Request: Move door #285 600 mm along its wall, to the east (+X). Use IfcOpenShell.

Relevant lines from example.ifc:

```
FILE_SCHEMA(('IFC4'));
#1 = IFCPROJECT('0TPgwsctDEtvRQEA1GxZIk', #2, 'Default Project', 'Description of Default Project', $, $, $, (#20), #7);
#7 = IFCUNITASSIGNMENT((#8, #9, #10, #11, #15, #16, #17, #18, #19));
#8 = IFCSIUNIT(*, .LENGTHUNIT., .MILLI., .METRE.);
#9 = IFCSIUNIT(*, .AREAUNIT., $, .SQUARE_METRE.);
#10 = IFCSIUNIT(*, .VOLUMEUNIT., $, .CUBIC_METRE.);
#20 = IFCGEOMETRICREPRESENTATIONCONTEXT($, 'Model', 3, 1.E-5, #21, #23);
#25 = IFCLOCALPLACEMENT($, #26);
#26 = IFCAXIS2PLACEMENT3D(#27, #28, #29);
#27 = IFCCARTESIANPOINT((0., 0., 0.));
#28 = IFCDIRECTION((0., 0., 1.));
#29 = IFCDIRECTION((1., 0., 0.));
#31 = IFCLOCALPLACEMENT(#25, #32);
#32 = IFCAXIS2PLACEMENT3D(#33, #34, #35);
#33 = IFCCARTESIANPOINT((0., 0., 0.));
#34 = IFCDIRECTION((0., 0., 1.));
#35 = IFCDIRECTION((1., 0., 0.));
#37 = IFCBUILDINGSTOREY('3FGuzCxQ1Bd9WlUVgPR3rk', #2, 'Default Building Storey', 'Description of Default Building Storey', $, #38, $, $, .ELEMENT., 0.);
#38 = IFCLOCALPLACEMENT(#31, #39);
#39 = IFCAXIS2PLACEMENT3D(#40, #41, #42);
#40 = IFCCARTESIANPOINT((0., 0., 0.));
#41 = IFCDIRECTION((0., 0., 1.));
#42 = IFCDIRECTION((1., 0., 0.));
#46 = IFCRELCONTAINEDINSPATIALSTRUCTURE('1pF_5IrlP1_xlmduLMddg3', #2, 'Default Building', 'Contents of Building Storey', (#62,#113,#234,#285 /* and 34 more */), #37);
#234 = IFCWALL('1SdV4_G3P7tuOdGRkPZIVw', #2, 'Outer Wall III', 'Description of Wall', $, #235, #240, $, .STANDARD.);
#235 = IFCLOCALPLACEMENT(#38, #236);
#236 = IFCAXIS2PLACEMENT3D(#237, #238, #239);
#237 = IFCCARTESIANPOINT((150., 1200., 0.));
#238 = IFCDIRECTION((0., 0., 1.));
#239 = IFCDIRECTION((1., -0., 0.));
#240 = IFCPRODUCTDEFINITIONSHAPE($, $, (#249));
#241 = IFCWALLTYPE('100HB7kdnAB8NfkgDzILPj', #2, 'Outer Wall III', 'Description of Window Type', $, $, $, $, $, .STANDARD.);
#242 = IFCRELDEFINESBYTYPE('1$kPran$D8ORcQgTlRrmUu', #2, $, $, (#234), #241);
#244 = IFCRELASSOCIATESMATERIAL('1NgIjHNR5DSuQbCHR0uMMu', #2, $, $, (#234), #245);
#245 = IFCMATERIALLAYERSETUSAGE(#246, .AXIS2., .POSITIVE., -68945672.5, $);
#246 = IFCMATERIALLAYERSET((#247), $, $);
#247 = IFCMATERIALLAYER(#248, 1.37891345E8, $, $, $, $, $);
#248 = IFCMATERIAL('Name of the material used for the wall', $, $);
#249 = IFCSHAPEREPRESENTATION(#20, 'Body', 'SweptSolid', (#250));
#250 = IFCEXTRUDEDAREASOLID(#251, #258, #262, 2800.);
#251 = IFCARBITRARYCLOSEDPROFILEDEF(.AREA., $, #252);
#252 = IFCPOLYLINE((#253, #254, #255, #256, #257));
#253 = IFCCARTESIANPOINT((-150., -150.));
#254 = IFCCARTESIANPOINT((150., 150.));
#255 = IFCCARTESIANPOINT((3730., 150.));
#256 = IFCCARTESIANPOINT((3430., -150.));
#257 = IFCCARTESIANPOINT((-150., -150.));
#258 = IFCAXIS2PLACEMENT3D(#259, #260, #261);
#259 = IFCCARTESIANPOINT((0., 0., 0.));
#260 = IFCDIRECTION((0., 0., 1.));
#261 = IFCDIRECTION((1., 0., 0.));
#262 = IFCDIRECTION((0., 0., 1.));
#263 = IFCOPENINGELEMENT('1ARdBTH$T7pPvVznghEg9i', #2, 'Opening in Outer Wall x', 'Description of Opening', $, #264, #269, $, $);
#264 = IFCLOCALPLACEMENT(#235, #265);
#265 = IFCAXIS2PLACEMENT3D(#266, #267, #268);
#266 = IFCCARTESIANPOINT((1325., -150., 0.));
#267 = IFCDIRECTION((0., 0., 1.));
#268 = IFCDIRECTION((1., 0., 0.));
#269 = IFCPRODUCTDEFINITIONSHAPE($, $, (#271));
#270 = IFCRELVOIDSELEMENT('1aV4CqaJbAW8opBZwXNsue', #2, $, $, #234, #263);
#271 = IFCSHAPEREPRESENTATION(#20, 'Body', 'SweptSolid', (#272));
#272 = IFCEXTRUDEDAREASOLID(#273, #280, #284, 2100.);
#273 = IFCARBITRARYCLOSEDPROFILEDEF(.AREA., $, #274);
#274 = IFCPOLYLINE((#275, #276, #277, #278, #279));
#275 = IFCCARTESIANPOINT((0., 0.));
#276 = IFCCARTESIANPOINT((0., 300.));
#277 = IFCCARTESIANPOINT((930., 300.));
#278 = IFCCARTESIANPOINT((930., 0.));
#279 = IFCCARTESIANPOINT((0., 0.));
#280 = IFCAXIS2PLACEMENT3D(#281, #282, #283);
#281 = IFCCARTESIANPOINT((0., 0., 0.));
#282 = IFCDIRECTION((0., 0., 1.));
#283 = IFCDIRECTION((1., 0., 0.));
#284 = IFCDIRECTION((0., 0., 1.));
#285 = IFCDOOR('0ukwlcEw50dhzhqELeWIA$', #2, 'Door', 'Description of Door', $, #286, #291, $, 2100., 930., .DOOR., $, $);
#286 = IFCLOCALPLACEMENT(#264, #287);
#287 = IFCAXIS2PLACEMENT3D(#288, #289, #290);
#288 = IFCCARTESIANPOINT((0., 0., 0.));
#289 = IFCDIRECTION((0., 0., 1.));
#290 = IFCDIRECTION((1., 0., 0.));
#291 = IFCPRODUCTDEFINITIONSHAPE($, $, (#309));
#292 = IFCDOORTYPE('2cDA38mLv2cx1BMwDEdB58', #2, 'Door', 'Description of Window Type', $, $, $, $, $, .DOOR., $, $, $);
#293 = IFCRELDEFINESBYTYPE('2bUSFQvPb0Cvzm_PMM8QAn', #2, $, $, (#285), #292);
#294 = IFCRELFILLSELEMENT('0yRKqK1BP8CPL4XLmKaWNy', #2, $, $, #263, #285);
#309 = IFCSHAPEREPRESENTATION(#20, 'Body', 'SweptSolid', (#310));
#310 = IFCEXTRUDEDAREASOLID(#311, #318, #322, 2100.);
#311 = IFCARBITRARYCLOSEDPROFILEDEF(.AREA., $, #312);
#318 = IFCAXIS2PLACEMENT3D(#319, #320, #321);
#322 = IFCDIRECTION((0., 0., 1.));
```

```python
import ifcopenshell
import ifcopenshell.api.geometry
import ifcopenshell.util.placement
import ifcopenshell.util.unit

model = ifcopenshell.open("example.ifc")
unit_scale = ifcopenshell.util.unit.calculate_unit_scale(model)

door = model.by_id(285)
opening = door.FillsVoids[0].RelatingOpeningElement
wall = opening.VoidsElements[0].RelatingBuildingElement

wall_matrix = ifcopenshell.util.placement.get_local_placement(wall.ObjectPlacement)
shift = wall_matrix[:3, 0] * 0.6 / unit_scale
before = ifcopenshell.util.placement.get_local_placement(door.ObjectPlacement)[:3, 3].copy()

# The door is placed relative to its opening, so it follows when the opening moves.
matrix = ifcopenshell.util.placement.get_local_placement(opening.ObjectPlacement)
matrix[:3, 3] += shift
ifcopenshell.api.geometry.edit_object_placement(
    model, product=opening, matrix=matrix, is_si=False, should_transform_children=True
)

after = ifcopenshell.util.placement.get_local_placement(door.ObjectPlacement)[:3, 3]
print("door moved by", (after - before).round(3) + 0.0)

model.write("example-out.ifc")
```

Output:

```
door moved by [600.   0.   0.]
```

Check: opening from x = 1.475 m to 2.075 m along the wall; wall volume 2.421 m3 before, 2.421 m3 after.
